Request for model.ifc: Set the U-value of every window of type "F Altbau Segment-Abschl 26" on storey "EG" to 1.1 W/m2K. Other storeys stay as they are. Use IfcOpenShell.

First a look at what the model holds.

```python
import ifcopenshell
import ifcopenshell.util.element

model = ifcopenshell.open("model.ifc")
print(model.schema)
storey = next(s for s in model.by_type("IfcBuildingStorey") if s.Name == "EG")
windows = [e for e in ifcopenshell.util.element.get_decomposition(storey) if e.is_a("IfcWindow")]
seen = {}
for e in windows:
    element_type = ifcopenshell.util.element.get_type(e)
    key = (element_type.Name if element_type != e and element_type else None, ifcopenshell.util.element.get_pset(e, "Pset_WindowCommon", "ThermalTransmittance"))
    seen[key] = seen.get(key, 0) + 1
for (name, value), count in sorted(seen.items(), key=str):
    print(count, "x", name, "|", value)
```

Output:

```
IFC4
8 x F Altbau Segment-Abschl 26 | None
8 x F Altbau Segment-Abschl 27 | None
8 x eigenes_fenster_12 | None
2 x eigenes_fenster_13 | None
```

```python
import ifcopenshell
import ifcopenshell.api.pset
import ifcopenshell.util.element

model = ifcopenshell.open("model.ifc")

storey = next(s for s in model.by_type("IfcBuildingStorey") if s.Name == "EG")
windows = [e for e in ifcopenshell.util.element.get_decomposition(storey) if e.is_a("IfcWindow")]

count = 0
for e in windows:
    element_type = ifcopenshell.util.element.get_type(e)
    if element_type in (None, e) or element_type.Name != "F Altbau Segment-Abschl 26":
        continue
    # add_pset returns the element's existing set when there is one.
    pset = ifcopenshell.api.pset.add_pset(model, product=e, name="Pset_WindowCommon")
    ifcopenshell.api.pset.edit_pset(model, pset=pset, properties={"ThermalTransmittance": 1.1})
    count += 1

print(count, "windows updated")

model.write("model_updated.ifc")
```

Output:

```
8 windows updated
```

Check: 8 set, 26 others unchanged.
